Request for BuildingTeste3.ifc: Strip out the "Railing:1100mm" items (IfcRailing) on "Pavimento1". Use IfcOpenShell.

First a look at what the model holds.

```python
import ifcopenshell
import ifcopenshell.util.element

model = ifcopenshell.open("BuildingTeste3.ifc")
print(model.schema)
storey = next(s for s in model.by_type("IfcBuildingStorey") if s.Name == "Pavimento1")
railings = [e for e in ifcopenshell.util.element.get_decomposition(storey) if e.is_a("IfcRailing")]
seen = {}
for e in railings:
    element_type = ifcopenshell.util.element.get_type(e)
    name = element_type.Name if element_type not in (None, e) else None
    seen[name] = seen.get(name, 0) + 1
for name, count in sorted(seen.items(), key=str):
    print(count, "x", name)
```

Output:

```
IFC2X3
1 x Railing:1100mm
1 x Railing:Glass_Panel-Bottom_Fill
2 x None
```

```python
import ifcopenshell
import ifcopenshell.api.root
import ifcopenshell.util.element

model = ifcopenshell.open("BuildingTeste3.ifc")

storey = next(s for s in model.by_type("IfcBuildingStorey") if s.Name == "Pavimento1")
railings = [e for e in ifcopenshell.util.element.get_decomposition(storey) if e.is_a("IfcRailing")]
targets = [e for e in railings if (t := ifcopenshell.util.element.get_type(e)) not in (None, e) and t.Name == "Railing:1100mm"]

for e in targets:
    ifcopenshell.api.root.remove_product(model, product=e)
print(len(targets), "removed")

model.write("BuildingTeste3_updated.ifc")
```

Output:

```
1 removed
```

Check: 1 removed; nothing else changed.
